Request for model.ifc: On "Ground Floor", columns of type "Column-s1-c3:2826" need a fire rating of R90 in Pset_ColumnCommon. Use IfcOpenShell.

First a look at what the model holds.

```python
import ifcopenshell
import ifcopenshell.util.element

model = ifcopenshell.open("model.ifc")
print(model.schema)
storey = next(s for s in model.by_type("IfcBuildingStorey") if s.Name == "Ground Floor")
columns = [e for e in ifcopenshell.util.element.get_decomposition(storey) if e.is_a("IfcColumn")]
seen = {}
for e in columns:
    element_type = ifcopenshell.util.element.get_type(e)
    key = (element_type.Name if element_type != e and element_type else None, ifcopenshell.util.element.get_pset(e, "Pset_ColumnCommon", "FireRating"))
    seen[key] = seen.get(key, 0) + 1
for (name, value), count in sorted(seen.items(), key=str):
    print(count, "x", name, "|", value)
```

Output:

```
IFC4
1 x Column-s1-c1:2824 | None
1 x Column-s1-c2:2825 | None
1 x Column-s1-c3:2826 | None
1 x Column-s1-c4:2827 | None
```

```python
import ifcopenshell
import ifcopenshell.api.pset
import ifcopenshell.util.element

model = ifcopenshell.open("model.ifc")

storey = next(s for s in model.by_type("IfcBuildingStorey") if s.Name == "Ground Floor")
columns = [e for e in ifcopenshell.util.element.get_decomposition(storey) if e.is_a("IfcColumn")]

count = 0
for e in columns:
    element_type = ifcopenshell.util.element.get_type(e)
    if element_type in (None, e) or element_type.Name != "Column-s1-c3:2826":
        continue
    # add_pset returns the element's existing set when there is one.
    pset = ifcopenshell.api.pset.add_pset(model, product=e, name="Pset_ColumnCommon")
    ifcopenshell.api.pset.edit_pset(model, pset=pset, properties={"FireRating": "R90"})
    count += 1

print(count, "columns updated")

model.write("model_edited.ifc")
```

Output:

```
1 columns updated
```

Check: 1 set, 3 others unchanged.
